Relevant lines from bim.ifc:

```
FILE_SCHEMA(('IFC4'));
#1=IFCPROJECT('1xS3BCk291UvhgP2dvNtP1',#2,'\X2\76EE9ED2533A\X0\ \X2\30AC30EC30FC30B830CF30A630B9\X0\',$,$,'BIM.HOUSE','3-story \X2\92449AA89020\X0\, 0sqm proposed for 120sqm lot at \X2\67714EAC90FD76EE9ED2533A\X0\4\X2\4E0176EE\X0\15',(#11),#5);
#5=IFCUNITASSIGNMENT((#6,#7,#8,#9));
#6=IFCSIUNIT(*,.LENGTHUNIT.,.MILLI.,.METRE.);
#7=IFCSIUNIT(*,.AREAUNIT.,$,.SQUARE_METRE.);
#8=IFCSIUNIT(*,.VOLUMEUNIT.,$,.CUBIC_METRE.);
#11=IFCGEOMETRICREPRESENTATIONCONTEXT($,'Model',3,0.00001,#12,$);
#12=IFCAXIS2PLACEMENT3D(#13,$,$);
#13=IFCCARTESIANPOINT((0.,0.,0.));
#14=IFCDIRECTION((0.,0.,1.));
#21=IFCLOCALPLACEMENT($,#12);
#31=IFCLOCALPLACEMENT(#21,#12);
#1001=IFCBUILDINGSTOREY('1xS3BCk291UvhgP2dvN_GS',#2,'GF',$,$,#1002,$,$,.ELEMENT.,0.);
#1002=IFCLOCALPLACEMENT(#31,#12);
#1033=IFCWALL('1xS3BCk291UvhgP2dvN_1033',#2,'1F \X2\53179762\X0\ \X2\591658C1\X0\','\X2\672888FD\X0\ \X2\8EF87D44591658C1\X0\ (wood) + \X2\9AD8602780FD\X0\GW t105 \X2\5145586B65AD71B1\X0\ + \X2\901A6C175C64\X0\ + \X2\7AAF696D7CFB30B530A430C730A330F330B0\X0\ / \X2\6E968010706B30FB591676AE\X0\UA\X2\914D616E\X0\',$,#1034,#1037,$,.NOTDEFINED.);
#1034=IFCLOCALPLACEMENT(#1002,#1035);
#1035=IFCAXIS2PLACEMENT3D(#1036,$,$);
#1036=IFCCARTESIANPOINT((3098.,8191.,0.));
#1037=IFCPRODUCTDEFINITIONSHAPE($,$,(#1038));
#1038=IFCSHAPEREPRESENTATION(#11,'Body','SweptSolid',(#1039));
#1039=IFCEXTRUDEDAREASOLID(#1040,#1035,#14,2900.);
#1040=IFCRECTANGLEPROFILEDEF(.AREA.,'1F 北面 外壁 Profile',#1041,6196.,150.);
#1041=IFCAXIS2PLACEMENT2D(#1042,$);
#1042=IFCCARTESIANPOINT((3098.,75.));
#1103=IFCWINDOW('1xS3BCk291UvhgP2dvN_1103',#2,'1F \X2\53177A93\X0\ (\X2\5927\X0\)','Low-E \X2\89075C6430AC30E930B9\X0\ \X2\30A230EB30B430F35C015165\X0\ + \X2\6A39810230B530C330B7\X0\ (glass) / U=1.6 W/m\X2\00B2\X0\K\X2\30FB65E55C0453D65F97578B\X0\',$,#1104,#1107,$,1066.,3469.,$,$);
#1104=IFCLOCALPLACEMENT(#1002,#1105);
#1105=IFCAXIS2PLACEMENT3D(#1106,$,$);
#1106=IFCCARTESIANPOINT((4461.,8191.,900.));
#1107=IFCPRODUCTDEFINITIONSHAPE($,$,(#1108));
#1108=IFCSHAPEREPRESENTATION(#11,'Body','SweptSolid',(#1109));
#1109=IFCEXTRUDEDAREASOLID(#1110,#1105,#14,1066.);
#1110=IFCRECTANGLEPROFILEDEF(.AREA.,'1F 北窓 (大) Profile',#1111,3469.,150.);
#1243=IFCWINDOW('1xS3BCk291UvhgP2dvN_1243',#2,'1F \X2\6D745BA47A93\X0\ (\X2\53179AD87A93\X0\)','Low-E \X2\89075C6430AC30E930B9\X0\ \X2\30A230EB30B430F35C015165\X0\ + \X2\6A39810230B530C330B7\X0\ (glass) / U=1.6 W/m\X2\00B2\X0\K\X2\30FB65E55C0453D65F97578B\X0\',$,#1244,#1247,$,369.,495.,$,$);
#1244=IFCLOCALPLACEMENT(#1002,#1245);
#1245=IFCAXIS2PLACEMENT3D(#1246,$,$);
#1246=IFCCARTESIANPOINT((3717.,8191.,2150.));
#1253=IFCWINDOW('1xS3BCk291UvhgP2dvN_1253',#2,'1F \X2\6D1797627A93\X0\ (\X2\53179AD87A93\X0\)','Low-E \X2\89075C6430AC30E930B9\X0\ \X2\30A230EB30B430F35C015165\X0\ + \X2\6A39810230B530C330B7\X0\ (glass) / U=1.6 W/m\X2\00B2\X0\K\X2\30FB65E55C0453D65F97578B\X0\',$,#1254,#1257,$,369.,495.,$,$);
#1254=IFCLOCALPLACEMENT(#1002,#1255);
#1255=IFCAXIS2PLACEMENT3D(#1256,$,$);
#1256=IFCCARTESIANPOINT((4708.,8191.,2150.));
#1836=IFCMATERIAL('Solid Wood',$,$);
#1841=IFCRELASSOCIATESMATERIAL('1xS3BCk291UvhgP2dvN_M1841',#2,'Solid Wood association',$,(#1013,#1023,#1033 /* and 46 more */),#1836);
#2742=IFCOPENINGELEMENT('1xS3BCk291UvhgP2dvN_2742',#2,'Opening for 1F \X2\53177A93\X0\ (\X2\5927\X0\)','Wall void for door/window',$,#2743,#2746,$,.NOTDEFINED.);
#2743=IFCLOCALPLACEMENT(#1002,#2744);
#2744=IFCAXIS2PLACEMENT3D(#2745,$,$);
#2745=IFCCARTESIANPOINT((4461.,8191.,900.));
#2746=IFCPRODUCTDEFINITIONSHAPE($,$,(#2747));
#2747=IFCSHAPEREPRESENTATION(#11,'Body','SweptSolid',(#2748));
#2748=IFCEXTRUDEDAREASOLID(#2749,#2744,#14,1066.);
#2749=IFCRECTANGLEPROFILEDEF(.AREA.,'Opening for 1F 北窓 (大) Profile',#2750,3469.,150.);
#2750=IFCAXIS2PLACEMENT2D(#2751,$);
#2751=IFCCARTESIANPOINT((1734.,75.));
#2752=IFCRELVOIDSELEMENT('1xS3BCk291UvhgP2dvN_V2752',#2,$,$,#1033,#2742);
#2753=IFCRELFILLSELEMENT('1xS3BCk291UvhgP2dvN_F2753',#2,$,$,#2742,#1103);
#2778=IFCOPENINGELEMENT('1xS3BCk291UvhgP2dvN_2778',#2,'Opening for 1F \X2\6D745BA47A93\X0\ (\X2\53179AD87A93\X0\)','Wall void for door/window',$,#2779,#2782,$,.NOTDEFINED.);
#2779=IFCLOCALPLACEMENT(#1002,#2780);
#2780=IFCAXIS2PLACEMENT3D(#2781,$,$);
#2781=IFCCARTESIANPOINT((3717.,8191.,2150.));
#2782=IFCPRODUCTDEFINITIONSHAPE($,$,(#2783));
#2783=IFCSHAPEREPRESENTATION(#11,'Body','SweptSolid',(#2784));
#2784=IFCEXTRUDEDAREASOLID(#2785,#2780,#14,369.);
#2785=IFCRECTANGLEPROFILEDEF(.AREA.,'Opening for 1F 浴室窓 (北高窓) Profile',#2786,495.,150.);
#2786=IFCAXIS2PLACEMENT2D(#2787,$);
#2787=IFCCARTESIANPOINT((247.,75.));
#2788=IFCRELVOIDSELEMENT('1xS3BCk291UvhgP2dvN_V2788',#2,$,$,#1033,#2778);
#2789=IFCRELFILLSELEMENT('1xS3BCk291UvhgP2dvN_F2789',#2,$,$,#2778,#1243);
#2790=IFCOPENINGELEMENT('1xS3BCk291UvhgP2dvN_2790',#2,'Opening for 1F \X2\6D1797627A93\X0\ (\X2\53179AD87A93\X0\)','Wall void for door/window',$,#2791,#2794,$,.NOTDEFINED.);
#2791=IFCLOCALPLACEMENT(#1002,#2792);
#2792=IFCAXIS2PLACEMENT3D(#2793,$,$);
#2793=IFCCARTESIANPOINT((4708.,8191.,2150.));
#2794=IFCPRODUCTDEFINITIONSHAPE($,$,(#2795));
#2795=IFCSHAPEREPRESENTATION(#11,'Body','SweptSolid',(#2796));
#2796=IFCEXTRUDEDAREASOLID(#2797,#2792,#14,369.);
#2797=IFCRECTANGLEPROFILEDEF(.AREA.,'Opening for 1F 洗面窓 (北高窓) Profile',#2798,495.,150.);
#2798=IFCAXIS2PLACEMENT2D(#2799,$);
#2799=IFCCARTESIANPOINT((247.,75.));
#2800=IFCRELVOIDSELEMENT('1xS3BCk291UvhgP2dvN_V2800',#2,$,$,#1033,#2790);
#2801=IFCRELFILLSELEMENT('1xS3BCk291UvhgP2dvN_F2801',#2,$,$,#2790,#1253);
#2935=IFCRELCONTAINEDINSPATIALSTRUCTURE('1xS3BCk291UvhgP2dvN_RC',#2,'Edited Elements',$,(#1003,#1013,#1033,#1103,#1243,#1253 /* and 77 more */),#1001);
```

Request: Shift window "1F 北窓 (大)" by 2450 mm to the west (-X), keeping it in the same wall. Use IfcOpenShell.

```python
import ifcopenshell
import ifcopenshell.api.geometry
import ifcopenshell.util.placement
import ifcopenshell.util.unit

model = ifcopenshell.open("bim.ifc")
unit_scale = ifcopenshell.util.unit.calculate_unit_scale(model)

window = model.by_id(1103)
opening = window.FillsVoids[0].RelatingOpeningElement
wall = opening.VoidsElements[0].RelatingBuildingElement

wall_matrix = ifcopenshell.util.placement.get_local_placement(wall.ObjectPlacement)
shift = wall_matrix[:3, 0] * -2.45 / unit_scale
before = ifcopenshell.util.placement.get_local_placement(window.ObjectPlacement)[:3, 3].copy()

# The window is not placed relative to its opening, so move both.
for product in (opening, window):
    matrix = ifcopenshell.util.placement.get_local_placement(product.ObjectPlacement)
    matrix[:3, 3] += shift
    ifcopenshell.api.geometry.edit_object_placement(model, product=product, matrix=matrix, is_si=False)

after = ifcopenshell.util.placement.get_local_placement(window.ObjectPlacement)[:3, 3]
print("window moved by", (after - before).round(3) + 0.0)

model.write("bim_rev.ifc")
```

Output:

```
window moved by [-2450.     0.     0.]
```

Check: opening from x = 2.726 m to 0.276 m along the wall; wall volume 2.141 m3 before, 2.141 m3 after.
